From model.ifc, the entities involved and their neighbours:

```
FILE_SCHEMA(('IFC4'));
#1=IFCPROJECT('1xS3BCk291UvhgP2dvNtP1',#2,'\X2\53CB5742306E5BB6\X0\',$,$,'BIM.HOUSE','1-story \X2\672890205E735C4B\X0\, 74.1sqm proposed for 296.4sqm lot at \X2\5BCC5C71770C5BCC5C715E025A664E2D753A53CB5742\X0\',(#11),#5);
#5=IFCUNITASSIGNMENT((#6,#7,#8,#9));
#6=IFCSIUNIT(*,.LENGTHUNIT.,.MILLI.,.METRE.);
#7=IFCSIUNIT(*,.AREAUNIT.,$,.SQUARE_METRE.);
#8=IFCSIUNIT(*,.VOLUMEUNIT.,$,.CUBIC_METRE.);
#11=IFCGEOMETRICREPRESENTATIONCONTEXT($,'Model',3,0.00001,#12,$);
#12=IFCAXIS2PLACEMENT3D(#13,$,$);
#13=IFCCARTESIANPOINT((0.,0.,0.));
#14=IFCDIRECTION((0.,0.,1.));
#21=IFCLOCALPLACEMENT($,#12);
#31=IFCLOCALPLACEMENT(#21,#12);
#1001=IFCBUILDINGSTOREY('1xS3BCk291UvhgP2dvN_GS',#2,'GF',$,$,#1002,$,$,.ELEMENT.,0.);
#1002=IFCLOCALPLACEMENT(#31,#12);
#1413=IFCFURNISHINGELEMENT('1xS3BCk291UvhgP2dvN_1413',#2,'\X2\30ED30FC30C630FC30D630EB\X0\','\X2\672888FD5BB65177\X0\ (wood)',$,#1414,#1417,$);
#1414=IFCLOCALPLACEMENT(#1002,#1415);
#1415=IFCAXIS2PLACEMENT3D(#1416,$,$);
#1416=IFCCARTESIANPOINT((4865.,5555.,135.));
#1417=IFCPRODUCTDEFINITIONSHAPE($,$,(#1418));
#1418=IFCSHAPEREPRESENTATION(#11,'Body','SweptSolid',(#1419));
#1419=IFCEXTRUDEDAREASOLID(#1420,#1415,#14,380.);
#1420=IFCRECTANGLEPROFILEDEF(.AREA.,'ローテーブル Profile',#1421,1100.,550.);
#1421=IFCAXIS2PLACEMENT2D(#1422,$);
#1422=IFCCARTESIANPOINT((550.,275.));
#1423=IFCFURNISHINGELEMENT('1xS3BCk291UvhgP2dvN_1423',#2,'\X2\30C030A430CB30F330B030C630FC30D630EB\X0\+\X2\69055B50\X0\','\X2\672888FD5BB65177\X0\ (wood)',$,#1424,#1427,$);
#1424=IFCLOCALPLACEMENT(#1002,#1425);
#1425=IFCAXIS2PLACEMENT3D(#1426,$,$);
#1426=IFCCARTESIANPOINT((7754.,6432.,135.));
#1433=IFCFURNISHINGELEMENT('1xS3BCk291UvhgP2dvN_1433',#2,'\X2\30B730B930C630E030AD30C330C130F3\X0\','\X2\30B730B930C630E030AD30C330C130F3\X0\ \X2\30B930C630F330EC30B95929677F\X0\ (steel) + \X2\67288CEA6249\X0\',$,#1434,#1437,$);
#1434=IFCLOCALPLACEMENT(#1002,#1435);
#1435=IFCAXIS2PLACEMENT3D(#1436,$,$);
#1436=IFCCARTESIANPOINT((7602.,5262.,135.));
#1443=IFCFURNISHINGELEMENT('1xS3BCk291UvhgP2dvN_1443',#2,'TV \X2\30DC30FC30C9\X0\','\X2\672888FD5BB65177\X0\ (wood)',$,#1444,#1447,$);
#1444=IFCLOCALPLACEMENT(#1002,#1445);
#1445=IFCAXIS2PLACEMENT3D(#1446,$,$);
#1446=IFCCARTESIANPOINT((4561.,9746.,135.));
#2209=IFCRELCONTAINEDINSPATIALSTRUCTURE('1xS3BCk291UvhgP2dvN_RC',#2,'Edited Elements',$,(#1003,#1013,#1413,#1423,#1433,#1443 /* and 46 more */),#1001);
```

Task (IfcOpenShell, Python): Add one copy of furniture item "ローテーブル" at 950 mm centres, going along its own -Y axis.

```python
import ifcopenshell
import ifcopenshell.api.geometry
import ifcopenshell.api.root
import ifcopenshell.util.element
import ifcopenshell.util.placement
import ifcopenshell.util.unit

model = ifcopenshell.open("model.ifc")
unit_scale = ifcopenshell.util.unit.calculate_unit_scale(model)


def reuse_history(source, copy):
    """copy_class also copies each property set's owner history, people and application; keep the originals."""
    for rel in copy.IsDefinedBy:
        if rel.is_a("IfcRelDefinesByProperties") and (history := rel.RelatingPropertyDefinition.OwnerHistory):
            rel.RelatingPropertyDefinition.OwnerHistory = source.OwnerHistory
            ifcopenshell.util.element.remove_deep2(model, history)


source = model.by_guid("1xS3BCk291UvhgP2dvN_1413")
base = ifcopenshell.util.placement.get_local_placement(source.ObjectPlacement)
step = -base[:3, 1] * 0.95 / unit_scale

for i in range(1, 2):
    copy = ifcopenshell.api.root.copy_class(model, product=source)
    copy.Representation = ifcopenshell.util.element.copy_deep(
        model, source.Representation, exclude=["IfcGeometricRepresentationContext", "IfcRepresentationMap"]
    )
    reuse_history(source, copy)
    matrix = base.copy()
    matrix[:3, 3] += i * step
    print("added at", matrix[:3, 3].round(3) + 0.0)
    ifcopenshell.api.geometry.edit_object_placement(model, product=copy, matrix=matrix, is_si=False)

model.write("model_v2.ifc")
```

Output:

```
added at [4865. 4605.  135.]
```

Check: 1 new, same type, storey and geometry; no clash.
